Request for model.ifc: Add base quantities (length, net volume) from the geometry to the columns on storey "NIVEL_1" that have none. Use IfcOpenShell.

First a look at what the model holds.

```python
import ifcopenshell
import ifcopenshell.util.element
import ifcopenshell.util.unit

model = ifcopenshell.open("model.ifc")
print(model.schema)
for unit_type in ("LENGTHUNIT", "AREAUNIT", "VOLUMEUNIT"):
    print(unit_type, ifcopenshell.util.unit.calculate_unit_scale(model, unit_type))
storey = next(s for s in model.by_type("IfcBuildingStorey") if s.Name == "NIVEL_1")
columns = [e for e in ifcopenshell.util.element.get_decomposition(storey) if e.is_a("IfcColumn")]
for e in sorted(columns, key=lambda e: e.id()):
    print(e.id(), e.is_a(), e.Name, list(ifcopenshell.util.element.get_psets(e, qtos_only=True)), sep=" | ")
```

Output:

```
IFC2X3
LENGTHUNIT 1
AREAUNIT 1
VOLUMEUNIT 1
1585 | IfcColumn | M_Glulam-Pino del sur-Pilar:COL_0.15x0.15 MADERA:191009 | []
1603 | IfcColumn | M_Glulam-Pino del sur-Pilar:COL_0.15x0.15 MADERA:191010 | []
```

```python
import ifcopenshell
import ifcopenshell.api.pset
import ifcopenshell.geom
import ifcopenshell.util.element
import ifcopenshell.util.shape
import ifcopenshell.util.unit

model = ifcopenshell.open("model.ifc")
unit_scale = ifcopenshell.util.unit.calculate_unit_scale(model)
volume_scale = ifcopenshell.util.unit.calculate_unit_scale(model, "VOLUMEUNIT")
settings = ifcopenshell.geom.settings()

storey = next(s for s in model.by_type("IfcBuildingStorey") if s.Name == "NIVEL_1")
columns = [e for e in ifcopenshell.util.element.get_decomposition(storey) if e.is_a("IfcColumn")]

for e in sorted(columns, key=lambda e: e.id()):
    if ifcopenshell.util.element.get_psets(e, qtos_only=True, should_inherit=False):
        continue
    # Geometry comes back in metres, in the element's own axes.
    shape = ifcopenshell.geom.create_shape(settings, e)
    values = {
        "Length": ifcopenshell.util.shape.get_z(shape.geometry) / unit_scale,
        "NetVolume": ifcopenshell.util.shape.get_volume(shape.geometry) / volume_scale,
    }
    qto = ifcopenshell.api.pset.add_qto(model, product=e, name="BaseQuantities")
    ifcopenshell.api.pset.edit_qto(model, qto=qto, properties=values)
    print(e.id(), {k: round(v, 3) for k, v in values.items()})

model.write("model-out.ifc")
```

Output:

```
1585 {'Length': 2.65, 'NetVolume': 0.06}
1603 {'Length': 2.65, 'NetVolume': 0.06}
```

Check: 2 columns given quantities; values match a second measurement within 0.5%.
